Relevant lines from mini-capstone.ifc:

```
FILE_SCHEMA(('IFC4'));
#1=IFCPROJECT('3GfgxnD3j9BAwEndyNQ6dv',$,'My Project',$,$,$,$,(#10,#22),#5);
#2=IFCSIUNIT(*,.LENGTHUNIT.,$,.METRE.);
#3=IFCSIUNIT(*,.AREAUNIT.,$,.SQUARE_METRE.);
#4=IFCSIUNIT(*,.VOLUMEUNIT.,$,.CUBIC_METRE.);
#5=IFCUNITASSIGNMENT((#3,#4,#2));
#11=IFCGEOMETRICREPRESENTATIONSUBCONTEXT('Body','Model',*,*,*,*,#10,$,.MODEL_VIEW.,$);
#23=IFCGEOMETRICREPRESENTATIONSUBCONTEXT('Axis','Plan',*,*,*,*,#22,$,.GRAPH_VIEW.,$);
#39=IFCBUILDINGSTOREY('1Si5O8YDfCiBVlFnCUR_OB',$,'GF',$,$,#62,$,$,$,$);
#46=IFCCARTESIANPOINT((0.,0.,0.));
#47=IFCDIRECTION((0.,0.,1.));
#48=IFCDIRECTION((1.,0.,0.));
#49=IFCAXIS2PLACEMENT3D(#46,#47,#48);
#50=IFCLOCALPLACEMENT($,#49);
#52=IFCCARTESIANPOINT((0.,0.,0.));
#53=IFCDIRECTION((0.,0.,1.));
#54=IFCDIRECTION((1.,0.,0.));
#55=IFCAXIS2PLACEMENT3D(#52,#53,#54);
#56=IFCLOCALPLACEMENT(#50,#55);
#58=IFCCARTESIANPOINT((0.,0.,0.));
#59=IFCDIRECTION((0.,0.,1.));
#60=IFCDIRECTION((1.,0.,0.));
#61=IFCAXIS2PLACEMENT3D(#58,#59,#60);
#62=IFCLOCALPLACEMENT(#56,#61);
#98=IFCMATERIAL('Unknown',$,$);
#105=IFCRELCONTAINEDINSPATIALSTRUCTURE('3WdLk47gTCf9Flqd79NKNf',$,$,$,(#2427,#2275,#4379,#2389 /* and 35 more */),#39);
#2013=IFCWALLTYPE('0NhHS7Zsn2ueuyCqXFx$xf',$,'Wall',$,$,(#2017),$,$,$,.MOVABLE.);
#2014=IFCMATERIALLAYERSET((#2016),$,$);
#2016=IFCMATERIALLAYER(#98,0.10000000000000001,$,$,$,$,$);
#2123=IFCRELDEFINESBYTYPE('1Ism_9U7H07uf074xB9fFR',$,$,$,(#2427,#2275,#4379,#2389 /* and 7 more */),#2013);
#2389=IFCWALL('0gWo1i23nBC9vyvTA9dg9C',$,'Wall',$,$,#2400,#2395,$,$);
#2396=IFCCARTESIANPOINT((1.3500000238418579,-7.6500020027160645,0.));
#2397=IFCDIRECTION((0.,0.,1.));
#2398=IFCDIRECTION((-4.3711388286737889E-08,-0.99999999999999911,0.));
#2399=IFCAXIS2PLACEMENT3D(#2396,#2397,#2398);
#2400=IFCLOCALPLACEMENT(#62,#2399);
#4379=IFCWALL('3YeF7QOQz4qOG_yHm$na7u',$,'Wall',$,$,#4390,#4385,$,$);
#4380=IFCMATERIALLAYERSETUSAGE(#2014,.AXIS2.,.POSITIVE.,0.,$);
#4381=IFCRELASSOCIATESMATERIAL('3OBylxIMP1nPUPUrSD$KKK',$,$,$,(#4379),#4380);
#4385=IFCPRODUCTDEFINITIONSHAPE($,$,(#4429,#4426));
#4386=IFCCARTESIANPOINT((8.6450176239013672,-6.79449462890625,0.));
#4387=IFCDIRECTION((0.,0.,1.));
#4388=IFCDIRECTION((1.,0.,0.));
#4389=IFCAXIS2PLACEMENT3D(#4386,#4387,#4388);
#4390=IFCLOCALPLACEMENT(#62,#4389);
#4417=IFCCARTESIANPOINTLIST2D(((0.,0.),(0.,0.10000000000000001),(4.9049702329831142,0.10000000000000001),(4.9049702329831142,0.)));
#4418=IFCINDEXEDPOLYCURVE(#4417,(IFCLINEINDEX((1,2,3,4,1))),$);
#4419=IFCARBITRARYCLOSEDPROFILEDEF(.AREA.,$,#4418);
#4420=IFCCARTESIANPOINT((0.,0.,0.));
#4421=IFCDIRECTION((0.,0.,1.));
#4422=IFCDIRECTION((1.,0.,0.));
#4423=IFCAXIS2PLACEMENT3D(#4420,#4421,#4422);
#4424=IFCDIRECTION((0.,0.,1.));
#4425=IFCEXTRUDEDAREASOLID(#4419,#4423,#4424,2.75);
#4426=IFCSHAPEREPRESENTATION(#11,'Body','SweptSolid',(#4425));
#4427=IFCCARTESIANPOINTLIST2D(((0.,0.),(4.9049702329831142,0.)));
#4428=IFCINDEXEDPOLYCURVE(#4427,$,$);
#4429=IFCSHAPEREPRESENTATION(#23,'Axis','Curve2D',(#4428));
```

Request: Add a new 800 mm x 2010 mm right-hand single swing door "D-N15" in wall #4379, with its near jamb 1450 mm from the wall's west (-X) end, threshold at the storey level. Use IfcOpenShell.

```python
import numpy as np
import ifcopenshell
import ifcopenshell.api.feature
import ifcopenshell.api.geometry
import ifcopenshell.api.root
import ifcopenshell.api.spatial
import ifcopenshell.geom
import ifcopenshell.util.element
import ifcopenshell.util.placement
import ifcopenshell.util.representation
import ifcopenshell.util.shape
import ifcopenshell.util.unit

model = ifcopenshell.open("mini-capstone.ifc")
unit_scale = ifcopenshell.util.unit.calculate_unit_scale(model)
settings = ifcopenshell.geom.settings()


def volume(element):
    """Net volume in cubic metres, openings subtracted."""
    shape = ifcopenshell.geom.create_shape(settings, element)
    return ifcopenshell.util.shape.get_volume(shape.geometry)


wall = model.by_guid("3YeF7QOQz4qOG_yHm$na7u")
storey = ifcopenshell.util.element.get_container(wall, ifc_class="IfcBuildingStorey")
context = ifcopenshell.util.representation.get_context(model, "Model", "Body", "MODEL_VIEW")
before = volume(wall)

width, height, from_end, sill = 0.8, 2.01, 1.45, 0.0  # metres

# The wall runs along its own X axis, and the end named is its -X end.
wall_shape = ifcopenshell.geom.create_shape(settings, wall)
x, y, z = ifcopenshell.util.shape.get_vertices(wall_shape.geometry).T
start = x.min() + from_end
face, thickness = float(y.min()), float(y.max() - y.min())
wall_matrix = ifcopenshell.util.placement.get_local_placement(wall.ObjectPlacement)
level = ifcopenshell.util.placement.get_local_placement(storey.ObjectPlacement)[2, 3]


def in_wall(x, y):
    """Placement at x, y metres in the wall's axes, at sill height."""
    matrix = wall_matrix.copy()
    matrix[:, 3] = wall_matrix @ np.array([x / unit_scale, y / unit_scale, 0.0, 1.0])
    matrix[2, 3] = level + sill / unit_scale
    return matrix


# Opening: a box that overshoots both wall faces by 50 mm.
opening = ifcopenshell.api.root.create_entity(model, ifc_class="IfcOpeningElement", predefined_type="OPENING")
box = ifcopenshell.api.geometry.add_wall_representation(
    model, context=context, length=width, height=height, thickness=thickness + 0.1
)
ifcopenshell.api.geometry.assign_representation(model, product=opening, representation=box)
ifcopenshell.api.geometry.edit_object_placement(model, product=opening, matrix=in_wall(start, face - 0.05), is_si=False)
ifcopenshell.api.feature.add_feature(model, feature=opening, element=wall)

door = ifcopenshell.api.root.create_entity(model, ifc_class="IfcDoor", name="D-N15", predefined_type="DOOR")
door.OverallWidth, door.OverallHeight = width / unit_scale, height / unit_scale
door.OperationType = "SINGLE_SWING_RIGHT"
body = ifcopenshell.api.geometry.add_door_representation(
    model,
    context=context,
    overall_width=door.OverallWidth,
    overall_height=door.OverallHeight,
    operation_type="SINGLE_SWING_RIGHT",
    lining_properties={"LiningDepth": thickness / unit_scale, "ThresholdDepth": thickness / unit_scale},
)
ifcopenshell.api.geometry.assign_representation(model, product=door, representation=body)
ifcopenshell.api.spatial.assign_container(model, products=[door], relating_structure=storey)
ifcopenshell.api.feature.add_filling(model, opening=opening, element=door)

# The lining spans the wall, so the door starts at the wall face.
ifcopenshell.api.geometry.edit_object_placement(model, product=door, matrix=in_wall(start, face), is_si=False)

after = volume(wall)

print(f"wall volume {before:.3f} -> {after:.3f} m3")

model.write("mini-capstone_edited.ifc")
```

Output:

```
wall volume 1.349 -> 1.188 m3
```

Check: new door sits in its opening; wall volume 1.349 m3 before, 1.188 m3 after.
